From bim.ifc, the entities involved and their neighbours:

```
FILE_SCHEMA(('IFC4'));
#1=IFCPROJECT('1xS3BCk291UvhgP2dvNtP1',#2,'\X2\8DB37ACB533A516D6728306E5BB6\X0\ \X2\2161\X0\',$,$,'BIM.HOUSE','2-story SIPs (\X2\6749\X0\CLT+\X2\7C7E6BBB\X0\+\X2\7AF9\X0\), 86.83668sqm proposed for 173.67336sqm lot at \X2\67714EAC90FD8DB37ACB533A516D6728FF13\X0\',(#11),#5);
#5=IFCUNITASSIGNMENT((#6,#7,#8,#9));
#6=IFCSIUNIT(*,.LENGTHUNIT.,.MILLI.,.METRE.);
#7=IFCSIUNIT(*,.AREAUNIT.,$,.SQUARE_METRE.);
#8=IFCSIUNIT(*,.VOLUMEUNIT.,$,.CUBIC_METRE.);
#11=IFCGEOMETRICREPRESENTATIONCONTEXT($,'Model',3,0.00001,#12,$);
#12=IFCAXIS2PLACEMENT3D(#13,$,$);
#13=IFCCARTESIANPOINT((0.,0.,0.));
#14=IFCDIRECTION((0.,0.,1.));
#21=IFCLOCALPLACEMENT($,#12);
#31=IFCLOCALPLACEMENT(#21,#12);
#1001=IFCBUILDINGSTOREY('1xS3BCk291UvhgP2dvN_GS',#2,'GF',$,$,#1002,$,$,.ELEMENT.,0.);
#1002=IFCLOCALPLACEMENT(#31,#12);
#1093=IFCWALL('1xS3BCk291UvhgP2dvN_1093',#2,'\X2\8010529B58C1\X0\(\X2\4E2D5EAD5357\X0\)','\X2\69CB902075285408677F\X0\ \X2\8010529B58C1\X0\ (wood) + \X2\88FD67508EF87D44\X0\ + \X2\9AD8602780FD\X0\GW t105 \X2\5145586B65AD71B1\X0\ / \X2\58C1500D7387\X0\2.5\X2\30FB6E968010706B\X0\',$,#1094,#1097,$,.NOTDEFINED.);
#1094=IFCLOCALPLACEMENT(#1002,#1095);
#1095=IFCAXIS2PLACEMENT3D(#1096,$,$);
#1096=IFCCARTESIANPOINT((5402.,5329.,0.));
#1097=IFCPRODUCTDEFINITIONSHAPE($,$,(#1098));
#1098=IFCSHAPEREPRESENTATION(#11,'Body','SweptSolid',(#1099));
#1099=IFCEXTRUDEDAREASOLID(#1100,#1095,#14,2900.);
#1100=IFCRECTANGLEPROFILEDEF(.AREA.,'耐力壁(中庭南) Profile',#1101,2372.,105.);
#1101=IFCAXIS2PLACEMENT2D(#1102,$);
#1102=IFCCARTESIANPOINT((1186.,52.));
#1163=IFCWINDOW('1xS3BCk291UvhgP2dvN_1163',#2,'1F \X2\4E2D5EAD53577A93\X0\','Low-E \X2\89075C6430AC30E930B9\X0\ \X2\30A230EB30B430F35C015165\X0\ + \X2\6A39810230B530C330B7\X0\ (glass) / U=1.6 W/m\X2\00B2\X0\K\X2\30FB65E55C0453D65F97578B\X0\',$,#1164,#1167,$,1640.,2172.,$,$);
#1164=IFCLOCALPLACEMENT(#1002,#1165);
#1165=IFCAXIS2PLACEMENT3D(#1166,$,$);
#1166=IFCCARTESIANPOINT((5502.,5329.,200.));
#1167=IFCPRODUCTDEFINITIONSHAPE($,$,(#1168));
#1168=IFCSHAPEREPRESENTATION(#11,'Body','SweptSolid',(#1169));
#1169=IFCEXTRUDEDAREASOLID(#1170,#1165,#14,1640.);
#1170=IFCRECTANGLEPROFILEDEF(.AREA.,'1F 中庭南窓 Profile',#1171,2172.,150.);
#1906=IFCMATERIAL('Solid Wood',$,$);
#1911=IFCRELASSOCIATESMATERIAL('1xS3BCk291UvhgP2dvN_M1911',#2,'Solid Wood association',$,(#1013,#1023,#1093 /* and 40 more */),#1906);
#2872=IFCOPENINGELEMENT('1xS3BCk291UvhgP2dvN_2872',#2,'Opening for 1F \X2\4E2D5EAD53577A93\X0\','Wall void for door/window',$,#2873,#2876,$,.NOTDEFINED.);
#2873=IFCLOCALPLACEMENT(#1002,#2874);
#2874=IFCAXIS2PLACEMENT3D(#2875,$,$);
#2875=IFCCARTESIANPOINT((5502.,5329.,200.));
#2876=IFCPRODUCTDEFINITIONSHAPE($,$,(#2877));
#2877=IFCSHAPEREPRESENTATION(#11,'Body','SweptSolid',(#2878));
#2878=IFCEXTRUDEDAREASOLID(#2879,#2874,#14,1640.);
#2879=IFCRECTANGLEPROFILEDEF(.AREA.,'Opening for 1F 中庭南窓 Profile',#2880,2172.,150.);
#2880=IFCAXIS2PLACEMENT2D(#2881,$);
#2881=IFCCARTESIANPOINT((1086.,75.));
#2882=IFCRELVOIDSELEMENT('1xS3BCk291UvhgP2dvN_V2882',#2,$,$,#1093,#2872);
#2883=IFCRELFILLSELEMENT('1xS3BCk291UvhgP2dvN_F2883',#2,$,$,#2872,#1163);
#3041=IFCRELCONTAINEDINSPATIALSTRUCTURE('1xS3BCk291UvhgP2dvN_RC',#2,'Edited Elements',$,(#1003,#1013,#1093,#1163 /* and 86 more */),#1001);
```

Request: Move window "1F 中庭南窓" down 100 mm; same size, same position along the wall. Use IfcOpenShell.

```python
import numpy as np
import ifcopenshell
import ifcopenshell.api.geometry
import ifcopenshell.util.placement
import ifcopenshell.util.unit

model = ifcopenshell.open("bim.ifc")
unit_scale = ifcopenshell.util.unit.calculate_unit_scale(model)

window = model.by_id(1163)
opening = window.FillsVoids[0].RelatingOpeningElement
dz = -0.1 / unit_scale

shift = np.array([0.0, 0.0, dz])
# The window is not placed relative to its opening, so move both.
for product in (opening, window):
    matrix = ifcopenshell.util.placement.get_local_placement(product.ObjectPlacement)
    matrix[:3, 3] += shift
    ifcopenshell.api.geometry.edit_object_placement(model, product=product, matrix=matrix, is_si=False)

print(f"moved by {dz * unit_scale:+.3f} m")

model.write("bim_updated.ifc")
```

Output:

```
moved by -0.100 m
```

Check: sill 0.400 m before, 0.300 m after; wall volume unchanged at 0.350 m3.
